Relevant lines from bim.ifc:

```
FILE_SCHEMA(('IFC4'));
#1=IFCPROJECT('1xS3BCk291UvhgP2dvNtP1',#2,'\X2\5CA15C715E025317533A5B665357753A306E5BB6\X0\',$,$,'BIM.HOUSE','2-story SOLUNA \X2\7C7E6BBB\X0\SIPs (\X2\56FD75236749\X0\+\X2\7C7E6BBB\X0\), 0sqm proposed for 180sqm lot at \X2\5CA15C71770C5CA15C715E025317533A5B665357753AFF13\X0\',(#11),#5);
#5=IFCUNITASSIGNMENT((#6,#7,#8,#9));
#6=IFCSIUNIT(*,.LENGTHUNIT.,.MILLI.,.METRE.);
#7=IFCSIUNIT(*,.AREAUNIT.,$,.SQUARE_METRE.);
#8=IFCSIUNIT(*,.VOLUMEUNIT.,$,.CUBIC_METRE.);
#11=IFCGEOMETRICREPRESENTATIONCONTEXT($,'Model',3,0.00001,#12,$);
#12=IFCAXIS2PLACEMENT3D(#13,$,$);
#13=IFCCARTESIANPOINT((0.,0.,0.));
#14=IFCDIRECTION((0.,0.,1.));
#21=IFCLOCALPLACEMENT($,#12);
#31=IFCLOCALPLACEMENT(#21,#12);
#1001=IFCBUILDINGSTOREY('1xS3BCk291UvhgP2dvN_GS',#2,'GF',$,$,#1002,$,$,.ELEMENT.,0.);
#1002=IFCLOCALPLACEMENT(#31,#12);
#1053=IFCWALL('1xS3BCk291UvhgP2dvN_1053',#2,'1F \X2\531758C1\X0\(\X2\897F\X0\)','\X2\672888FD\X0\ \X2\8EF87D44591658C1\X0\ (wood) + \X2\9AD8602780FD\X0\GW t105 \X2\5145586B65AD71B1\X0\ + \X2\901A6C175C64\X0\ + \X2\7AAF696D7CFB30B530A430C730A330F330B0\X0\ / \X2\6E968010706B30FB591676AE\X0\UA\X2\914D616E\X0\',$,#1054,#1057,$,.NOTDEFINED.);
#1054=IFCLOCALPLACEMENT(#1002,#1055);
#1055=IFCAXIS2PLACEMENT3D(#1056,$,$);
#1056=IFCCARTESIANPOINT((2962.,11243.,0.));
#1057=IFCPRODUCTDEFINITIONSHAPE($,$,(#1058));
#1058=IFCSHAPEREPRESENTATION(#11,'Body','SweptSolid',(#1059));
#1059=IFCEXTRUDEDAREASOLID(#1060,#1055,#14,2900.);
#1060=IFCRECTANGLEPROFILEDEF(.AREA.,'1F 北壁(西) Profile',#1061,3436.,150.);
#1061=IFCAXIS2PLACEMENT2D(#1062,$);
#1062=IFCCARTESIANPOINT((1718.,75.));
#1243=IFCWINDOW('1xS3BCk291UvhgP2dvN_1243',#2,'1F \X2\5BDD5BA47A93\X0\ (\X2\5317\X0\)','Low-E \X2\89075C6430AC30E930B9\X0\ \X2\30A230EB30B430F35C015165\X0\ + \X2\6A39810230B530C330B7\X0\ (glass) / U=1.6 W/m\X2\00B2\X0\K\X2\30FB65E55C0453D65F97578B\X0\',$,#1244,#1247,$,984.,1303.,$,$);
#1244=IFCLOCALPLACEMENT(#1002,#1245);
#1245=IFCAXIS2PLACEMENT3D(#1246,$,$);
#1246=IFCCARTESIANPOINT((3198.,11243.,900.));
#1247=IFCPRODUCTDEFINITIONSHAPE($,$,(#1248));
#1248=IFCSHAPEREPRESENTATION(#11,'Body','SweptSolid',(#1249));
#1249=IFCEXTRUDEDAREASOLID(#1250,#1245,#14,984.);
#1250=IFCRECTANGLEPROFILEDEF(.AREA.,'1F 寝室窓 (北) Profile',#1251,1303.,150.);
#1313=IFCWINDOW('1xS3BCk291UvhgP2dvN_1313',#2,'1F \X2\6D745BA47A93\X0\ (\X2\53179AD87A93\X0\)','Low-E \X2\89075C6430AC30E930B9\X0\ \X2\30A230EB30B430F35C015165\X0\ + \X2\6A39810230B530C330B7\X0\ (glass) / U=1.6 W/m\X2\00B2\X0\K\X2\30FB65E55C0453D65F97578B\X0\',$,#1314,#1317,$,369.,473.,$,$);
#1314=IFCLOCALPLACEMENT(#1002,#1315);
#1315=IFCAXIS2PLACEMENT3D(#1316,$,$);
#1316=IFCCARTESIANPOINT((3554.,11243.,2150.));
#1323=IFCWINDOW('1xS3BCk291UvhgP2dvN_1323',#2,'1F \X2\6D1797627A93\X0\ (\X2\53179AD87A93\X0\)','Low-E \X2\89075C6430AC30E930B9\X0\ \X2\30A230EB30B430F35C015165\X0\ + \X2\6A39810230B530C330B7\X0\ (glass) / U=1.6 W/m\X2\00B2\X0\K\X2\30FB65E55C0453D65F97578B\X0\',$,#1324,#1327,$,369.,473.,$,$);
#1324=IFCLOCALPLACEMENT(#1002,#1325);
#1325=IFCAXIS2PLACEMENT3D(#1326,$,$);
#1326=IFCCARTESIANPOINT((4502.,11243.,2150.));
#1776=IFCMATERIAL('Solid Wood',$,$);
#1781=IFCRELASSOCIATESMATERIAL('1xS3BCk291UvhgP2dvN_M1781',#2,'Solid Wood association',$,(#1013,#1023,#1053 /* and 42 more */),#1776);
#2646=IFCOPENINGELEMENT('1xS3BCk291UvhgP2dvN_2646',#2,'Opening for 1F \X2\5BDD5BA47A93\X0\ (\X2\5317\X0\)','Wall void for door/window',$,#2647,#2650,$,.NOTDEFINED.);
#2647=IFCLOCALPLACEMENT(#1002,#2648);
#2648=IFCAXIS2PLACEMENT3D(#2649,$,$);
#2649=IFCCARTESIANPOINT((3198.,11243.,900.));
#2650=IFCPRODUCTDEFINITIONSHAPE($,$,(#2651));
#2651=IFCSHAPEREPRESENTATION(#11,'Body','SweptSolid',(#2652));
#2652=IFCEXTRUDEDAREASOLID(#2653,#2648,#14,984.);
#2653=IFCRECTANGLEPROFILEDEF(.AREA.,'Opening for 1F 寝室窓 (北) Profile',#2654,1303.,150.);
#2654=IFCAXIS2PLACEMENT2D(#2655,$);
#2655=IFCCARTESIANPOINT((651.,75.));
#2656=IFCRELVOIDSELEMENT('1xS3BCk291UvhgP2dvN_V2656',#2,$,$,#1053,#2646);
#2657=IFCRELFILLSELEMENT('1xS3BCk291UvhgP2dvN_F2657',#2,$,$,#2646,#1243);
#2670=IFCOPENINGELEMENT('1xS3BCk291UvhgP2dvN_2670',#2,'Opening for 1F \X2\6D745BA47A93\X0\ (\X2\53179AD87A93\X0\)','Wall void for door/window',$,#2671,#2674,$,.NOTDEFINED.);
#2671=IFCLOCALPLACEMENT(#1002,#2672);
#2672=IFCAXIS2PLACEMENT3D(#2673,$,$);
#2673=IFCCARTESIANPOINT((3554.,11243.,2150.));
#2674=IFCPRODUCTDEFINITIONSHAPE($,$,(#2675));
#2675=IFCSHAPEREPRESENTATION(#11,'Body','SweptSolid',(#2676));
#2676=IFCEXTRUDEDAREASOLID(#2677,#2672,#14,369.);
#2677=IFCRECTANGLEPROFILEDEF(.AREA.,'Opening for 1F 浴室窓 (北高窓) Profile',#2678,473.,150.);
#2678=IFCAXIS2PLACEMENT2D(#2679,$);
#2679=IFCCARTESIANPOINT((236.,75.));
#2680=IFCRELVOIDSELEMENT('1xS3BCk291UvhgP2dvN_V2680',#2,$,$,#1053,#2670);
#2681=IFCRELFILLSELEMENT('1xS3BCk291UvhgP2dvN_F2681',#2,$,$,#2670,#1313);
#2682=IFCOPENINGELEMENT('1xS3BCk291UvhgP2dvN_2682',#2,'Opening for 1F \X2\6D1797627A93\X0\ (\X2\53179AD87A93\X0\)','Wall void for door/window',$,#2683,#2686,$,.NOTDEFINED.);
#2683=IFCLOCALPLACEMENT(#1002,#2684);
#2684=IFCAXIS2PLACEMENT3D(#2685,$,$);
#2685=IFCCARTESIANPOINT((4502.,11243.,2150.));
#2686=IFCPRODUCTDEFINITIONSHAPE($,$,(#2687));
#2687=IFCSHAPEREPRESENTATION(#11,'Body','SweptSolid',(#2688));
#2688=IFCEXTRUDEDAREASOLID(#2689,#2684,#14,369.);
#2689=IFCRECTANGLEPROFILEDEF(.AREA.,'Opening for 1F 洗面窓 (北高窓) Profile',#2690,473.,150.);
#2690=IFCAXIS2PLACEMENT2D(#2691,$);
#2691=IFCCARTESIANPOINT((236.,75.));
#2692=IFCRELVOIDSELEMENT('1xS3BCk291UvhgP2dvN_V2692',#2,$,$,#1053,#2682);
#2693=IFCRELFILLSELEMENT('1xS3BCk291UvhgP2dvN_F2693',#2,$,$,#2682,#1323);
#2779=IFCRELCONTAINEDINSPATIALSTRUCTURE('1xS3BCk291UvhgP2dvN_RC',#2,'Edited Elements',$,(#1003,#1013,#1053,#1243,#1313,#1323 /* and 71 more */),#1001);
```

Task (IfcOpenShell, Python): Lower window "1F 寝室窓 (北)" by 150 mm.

```python
import numpy as np
import ifcopenshell
import ifcopenshell.api.geometry
import ifcopenshell.util.placement
import ifcopenshell.util.unit

model = ifcopenshell.open("bim.ifc")
unit_scale = ifcopenshell.util.unit.calculate_unit_scale(model)

window = model.by_id(1243)
opening = window.FillsVoids[0].RelatingOpeningElement
dz = -0.15 / unit_scale

shift = np.array([0.0, 0.0, dz])
# The window is not placed relative to its opening, so move both.
for product in (opening, window):
    matrix = ifcopenshell.util.placement.get_local_placement(product.ObjectPlacement)
    matrix[:3, 3] += shift
    ifcopenshell.api.geometry.edit_object_placement(model, product=product, matrix=matrix, is_si=False)

print(f"moved by {dz * unit_scale:+.3f} m")

model.write("bim_updated.ifc")
```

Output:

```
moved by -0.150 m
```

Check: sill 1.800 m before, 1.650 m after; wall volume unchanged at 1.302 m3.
